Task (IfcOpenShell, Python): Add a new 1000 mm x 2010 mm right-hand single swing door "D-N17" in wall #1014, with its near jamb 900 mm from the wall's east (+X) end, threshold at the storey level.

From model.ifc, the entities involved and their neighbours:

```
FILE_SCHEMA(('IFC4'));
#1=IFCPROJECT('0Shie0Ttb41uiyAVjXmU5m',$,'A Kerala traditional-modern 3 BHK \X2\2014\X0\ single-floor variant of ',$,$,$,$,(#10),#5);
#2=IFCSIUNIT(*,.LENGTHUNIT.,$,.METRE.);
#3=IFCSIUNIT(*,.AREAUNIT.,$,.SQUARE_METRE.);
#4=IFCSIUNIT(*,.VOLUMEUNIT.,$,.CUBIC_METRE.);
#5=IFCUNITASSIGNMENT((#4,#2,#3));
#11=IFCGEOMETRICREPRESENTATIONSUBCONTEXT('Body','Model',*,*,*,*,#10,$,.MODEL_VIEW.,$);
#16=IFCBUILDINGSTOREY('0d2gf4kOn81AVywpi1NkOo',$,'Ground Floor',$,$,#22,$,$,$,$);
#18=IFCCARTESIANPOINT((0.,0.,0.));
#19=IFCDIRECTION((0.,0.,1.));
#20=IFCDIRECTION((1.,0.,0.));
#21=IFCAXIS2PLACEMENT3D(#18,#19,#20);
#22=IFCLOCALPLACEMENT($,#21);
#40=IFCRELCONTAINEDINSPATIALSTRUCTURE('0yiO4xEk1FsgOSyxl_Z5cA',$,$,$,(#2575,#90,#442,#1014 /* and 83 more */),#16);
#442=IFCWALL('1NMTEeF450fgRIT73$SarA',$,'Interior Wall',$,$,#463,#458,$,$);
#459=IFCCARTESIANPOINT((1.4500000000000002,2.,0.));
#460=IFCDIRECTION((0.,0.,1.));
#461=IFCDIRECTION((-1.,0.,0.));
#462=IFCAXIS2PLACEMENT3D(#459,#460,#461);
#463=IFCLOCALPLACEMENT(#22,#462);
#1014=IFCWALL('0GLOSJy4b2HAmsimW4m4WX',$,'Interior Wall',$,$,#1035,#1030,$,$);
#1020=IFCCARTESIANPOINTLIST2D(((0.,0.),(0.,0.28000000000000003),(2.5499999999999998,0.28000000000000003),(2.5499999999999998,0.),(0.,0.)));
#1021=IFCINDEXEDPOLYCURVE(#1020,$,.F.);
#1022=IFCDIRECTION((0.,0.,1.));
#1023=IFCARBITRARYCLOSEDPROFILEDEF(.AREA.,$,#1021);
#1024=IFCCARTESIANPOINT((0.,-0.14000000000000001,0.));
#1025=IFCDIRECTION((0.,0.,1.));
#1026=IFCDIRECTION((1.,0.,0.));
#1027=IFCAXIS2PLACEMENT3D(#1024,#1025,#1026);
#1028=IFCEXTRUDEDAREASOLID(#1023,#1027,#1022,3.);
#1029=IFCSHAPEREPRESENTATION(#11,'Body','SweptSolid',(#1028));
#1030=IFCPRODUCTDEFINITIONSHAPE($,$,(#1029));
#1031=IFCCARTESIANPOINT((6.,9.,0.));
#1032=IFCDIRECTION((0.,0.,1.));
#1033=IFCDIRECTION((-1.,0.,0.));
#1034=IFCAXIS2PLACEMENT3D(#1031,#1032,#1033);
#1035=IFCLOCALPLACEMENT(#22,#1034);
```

```python
import numpy as np
import ifcopenshell
import ifcopenshell.api.feature
import ifcopenshell.api.geometry
import ifcopenshell.api.root
import ifcopenshell.api.spatial
import ifcopenshell.geom
import ifcopenshell.util.element
import ifcopenshell.util.placement
import ifcopenshell.util.representation
import ifcopenshell.util.shape
import ifcopenshell.util.unit

model = ifcopenshell.open("model.ifc")
unit_scale = ifcopenshell.util.unit.calculate_unit_scale(model)
settings = ifcopenshell.geom.settings()


def volume(element):
    """Net volume in cubic metres, openings subtracted."""
    shape = ifcopenshell.geom.create_shape(settings, element)
    return ifcopenshell.util.shape.get_volume(shape.geometry)


wall = model.by_id(1014)
storey = ifcopenshell.util.element.get_container(wall, ifc_class="IfcBuildingStorey")
context = ifcopenshell.util.representation.get_context(model, "Model", "Body", "MODEL_VIEW")
before = volume(wall)

width, height, from_end, sill = 1, 2.01, 0.9, 0.0  # metres

# The wall runs along its own X axis, and the end named is its -X end.
wall_shape = ifcopenshell.geom.create_shape(settings, wall)
x, y, z = ifcopenshell.util.shape.get_vertices(wall_shape.geometry).T
start = x.min() + from_end
face, thickness = float(y.min()), float(y.max() - y.min())
wall_matrix = ifcopenshell.util.placement.get_local_placement(wall.ObjectPlacement)
level = ifcopenshell.util.placement.get_local_placement(storey.ObjectPlacement)[2, 3]


def in_wall(x, y):
    """Placement at x, y metres in the wall's axes, at sill height."""
    matrix = wall_matrix.copy()
    matrix[:, 3] = wall_matrix @ np.array([x / unit_scale, y / unit_scale, 0.0, 1.0])
    matrix[2, 3] = level + sill / unit_scale
    return matrix


# Opening: a box that overshoots both wall faces by 50 mm.
opening = ifcopenshell.api.root.create_entity(model, ifc_class="IfcOpeningElement", predefined_type="OPENING")
box = ifcopenshell.api.geometry.add_wall_representation(
    model, context=context, length=width, height=height, thickness=thickness + 0.1
)
ifcopenshell.api.geometry.assign_representation(model, product=opening, representation=box)
ifcopenshell.api.geometry.edit_object_placement(model, product=opening, matrix=in_wall(start, face - 0.05), is_si=False)
ifcopenshell.api.feature.add_feature(model, feature=opening, element=wall)

door = ifcopenshell.api.root.create_entity(model, ifc_class="IfcDoor", name="D-N17", predefined_type="DOOR")
door.OverallWidth, door.OverallHeight = width / unit_scale, height / unit_scale
door.OperationType = "SINGLE_SWING_RIGHT"
body = ifcopenshell.api.geometry.add_door_representation(
    model,
    context=context,
    overall_width=door.OverallWidth,
    overall_height=door.OverallHeight,
    operation_type="SINGLE_SWING_RIGHT",
    lining_properties={"LiningDepth": thickness / unit_scale, "ThresholdDepth": thickness / unit_scale},
)
ifcopenshell.api.geometry.assign_representation(model, product=door, representation=body)
ifcopenshell.api.spatial.assign_container(model, products=[door], relating_structure=storey)
ifcopenshell.api.feature.add_filling(model, opening=opening, element=door)

# The lining spans the wall, so the door starts at the wall face.
ifcopenshell.api.geometry.edit_object_placement(model, product=door, matrix=in_wall(start, face), is_si=False)

after = volume(wall)

print(f"wall volume {before:.3f} -> {after:.3f} m3")

model.write("model_rev.ifc")
```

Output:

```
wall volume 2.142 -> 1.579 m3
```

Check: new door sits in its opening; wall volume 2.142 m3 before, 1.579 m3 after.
